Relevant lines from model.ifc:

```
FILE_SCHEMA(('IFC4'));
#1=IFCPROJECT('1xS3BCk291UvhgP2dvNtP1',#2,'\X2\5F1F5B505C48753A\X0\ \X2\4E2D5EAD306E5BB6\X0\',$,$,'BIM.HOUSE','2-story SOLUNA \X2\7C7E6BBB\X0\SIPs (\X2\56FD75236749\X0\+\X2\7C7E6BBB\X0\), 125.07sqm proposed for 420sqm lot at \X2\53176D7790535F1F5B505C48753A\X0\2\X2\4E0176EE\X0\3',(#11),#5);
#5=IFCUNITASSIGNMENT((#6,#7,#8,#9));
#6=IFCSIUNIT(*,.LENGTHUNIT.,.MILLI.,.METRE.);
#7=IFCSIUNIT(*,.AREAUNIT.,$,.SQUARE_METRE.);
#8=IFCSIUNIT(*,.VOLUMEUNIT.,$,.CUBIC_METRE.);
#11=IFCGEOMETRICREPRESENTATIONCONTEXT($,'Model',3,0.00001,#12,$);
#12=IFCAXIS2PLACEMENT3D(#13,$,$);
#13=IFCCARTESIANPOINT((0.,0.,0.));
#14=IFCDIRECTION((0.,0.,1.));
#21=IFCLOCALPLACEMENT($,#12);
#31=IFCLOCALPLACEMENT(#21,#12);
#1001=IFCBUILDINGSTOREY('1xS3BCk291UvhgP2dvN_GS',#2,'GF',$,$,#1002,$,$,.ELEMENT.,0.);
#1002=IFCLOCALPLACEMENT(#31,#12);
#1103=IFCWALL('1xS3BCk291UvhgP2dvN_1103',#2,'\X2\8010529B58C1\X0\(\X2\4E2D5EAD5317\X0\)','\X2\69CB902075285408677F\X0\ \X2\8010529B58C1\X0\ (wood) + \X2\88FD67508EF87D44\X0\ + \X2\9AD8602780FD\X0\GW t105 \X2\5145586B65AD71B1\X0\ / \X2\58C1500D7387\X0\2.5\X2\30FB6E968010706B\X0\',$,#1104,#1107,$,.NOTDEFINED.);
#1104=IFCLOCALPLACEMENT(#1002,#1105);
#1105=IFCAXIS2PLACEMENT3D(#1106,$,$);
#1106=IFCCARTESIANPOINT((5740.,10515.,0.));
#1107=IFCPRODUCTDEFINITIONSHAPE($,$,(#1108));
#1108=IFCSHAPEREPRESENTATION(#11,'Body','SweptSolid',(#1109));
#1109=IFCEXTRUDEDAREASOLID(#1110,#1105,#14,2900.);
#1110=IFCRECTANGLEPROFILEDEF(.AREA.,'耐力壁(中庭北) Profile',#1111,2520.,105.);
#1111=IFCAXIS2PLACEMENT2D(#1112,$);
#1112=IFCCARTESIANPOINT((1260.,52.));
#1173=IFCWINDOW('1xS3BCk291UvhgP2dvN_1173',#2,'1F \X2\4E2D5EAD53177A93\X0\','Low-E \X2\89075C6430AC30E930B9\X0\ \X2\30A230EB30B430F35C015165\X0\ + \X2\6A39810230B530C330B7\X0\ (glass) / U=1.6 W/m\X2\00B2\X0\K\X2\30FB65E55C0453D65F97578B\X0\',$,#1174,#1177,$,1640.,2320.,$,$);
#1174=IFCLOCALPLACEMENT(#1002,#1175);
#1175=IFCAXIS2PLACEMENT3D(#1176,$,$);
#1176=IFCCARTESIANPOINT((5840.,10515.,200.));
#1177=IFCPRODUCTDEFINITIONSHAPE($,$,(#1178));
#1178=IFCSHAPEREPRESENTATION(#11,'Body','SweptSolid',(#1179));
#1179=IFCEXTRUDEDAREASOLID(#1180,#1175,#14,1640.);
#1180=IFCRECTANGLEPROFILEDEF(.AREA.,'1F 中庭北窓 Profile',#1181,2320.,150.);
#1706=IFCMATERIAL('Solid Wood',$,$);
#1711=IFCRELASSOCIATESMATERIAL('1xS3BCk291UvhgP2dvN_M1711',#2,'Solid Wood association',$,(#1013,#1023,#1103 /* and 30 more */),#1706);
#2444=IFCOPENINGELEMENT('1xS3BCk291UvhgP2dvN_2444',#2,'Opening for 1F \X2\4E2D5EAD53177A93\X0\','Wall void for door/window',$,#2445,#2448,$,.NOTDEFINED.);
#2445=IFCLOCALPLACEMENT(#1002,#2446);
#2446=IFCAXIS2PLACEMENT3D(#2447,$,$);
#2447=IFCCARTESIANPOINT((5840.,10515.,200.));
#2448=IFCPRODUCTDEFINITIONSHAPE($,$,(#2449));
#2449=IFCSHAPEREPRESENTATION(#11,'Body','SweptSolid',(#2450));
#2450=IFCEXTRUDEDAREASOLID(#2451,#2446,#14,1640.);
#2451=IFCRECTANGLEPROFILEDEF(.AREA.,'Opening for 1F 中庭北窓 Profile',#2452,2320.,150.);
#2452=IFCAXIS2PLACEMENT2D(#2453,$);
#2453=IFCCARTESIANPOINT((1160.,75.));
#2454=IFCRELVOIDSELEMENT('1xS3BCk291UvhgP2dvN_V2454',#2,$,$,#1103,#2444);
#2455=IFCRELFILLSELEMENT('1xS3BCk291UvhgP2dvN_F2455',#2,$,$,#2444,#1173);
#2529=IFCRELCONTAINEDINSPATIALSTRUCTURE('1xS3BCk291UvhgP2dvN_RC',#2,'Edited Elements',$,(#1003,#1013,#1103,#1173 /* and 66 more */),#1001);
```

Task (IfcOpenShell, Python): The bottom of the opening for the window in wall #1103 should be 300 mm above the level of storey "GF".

```python
import numpy as np
import ifcopenshell
import ifcopenshell.api.geometry
import ifcopenshell.geom
import ifcopenshell.util.element
import ifcopenshell.util.placement
import ifcopenshell.util.shape
import ifcopenshell.util.unit

model = ifcopenshell.open("model.ifc")
unit_scale = ifcopenshell.util.unit.calculate_unit_scale(model)

window = model.by_guid("1xS3BCk291UvhgP2dvN_1173")
opening = window.FillsVoids[0].RelatingOpeningElement
storey = ifcopenshell.util.element.get_container(window, ifc_class="IfcBuildingStorey")
level = ifcopenshell.util.placement.get_local_placement(storey.ObjectPlacement)[2, 3]

# The opening's origin need not be at the sill, so measure its lowest point.
shape = ifcopenshell.geom.create_shape(ifcopenshell.geom.settings(), opening)
bottom = ifcopenshell.util.shape.get_shape_bottom_elevation(shape, shape.geometry) / unit_scale
dz = level + 0.3 / unit_scale - bottom

shift = np.array([0.0, 0.0, dz])
# The window is not placed relative to its opening, so move both.
for product in (opening, window):
    matrix = ifcopenshell.util.placement.get_local_placement(product.ObjectPlacement)
    matrix[:3, 3] += shift
    ifcopenshell.api.geometry.edit_object_placement(model, product=product, matrix=matrix, is_si=False)

print(f"moved by {dz * unit_scale:+.3f} m")

model.write("model_edited.ifc")
```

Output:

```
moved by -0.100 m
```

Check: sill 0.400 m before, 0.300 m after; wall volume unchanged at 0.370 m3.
